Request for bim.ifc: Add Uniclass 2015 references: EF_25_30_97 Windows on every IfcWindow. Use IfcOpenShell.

First a look at what the model holds.

```python
import ifcopenshell

model = ifcopenshell.open("bim.ifc")
print(model.schema)
print("classifications:", [c.Name for c in model.by_type("IfcClassification")])
for ifc_class in ("IfcDoor", "IfcRoof", "IfcStair", "IfcWall", "IfcWindow"):
    print(ifc_class, len(model.by_type(ifc_class)))
```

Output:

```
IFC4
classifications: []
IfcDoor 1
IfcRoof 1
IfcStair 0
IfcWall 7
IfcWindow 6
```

```python
import ifcopenshell
import ifcopenshell.api.classification

model = ifcopenshell.open("bim.ifc")

system = ifcopenshell.api.classification.add_classification(model, classification="Uniclass 2015")

codes = {
    "IfcWindow": ("EF_25_30_97", "Windows"),
}
for ifc_class, (code, name) in codes.items():
    products = model.by_type(ifc_class)
    ifcopenshell.api.classification.add_reference(
        model, products=products, classification=system, identification=code, name=name
    )
    print(code, len(products))

model.write("bim_updated.ifc")
```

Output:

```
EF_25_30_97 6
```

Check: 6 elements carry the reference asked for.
